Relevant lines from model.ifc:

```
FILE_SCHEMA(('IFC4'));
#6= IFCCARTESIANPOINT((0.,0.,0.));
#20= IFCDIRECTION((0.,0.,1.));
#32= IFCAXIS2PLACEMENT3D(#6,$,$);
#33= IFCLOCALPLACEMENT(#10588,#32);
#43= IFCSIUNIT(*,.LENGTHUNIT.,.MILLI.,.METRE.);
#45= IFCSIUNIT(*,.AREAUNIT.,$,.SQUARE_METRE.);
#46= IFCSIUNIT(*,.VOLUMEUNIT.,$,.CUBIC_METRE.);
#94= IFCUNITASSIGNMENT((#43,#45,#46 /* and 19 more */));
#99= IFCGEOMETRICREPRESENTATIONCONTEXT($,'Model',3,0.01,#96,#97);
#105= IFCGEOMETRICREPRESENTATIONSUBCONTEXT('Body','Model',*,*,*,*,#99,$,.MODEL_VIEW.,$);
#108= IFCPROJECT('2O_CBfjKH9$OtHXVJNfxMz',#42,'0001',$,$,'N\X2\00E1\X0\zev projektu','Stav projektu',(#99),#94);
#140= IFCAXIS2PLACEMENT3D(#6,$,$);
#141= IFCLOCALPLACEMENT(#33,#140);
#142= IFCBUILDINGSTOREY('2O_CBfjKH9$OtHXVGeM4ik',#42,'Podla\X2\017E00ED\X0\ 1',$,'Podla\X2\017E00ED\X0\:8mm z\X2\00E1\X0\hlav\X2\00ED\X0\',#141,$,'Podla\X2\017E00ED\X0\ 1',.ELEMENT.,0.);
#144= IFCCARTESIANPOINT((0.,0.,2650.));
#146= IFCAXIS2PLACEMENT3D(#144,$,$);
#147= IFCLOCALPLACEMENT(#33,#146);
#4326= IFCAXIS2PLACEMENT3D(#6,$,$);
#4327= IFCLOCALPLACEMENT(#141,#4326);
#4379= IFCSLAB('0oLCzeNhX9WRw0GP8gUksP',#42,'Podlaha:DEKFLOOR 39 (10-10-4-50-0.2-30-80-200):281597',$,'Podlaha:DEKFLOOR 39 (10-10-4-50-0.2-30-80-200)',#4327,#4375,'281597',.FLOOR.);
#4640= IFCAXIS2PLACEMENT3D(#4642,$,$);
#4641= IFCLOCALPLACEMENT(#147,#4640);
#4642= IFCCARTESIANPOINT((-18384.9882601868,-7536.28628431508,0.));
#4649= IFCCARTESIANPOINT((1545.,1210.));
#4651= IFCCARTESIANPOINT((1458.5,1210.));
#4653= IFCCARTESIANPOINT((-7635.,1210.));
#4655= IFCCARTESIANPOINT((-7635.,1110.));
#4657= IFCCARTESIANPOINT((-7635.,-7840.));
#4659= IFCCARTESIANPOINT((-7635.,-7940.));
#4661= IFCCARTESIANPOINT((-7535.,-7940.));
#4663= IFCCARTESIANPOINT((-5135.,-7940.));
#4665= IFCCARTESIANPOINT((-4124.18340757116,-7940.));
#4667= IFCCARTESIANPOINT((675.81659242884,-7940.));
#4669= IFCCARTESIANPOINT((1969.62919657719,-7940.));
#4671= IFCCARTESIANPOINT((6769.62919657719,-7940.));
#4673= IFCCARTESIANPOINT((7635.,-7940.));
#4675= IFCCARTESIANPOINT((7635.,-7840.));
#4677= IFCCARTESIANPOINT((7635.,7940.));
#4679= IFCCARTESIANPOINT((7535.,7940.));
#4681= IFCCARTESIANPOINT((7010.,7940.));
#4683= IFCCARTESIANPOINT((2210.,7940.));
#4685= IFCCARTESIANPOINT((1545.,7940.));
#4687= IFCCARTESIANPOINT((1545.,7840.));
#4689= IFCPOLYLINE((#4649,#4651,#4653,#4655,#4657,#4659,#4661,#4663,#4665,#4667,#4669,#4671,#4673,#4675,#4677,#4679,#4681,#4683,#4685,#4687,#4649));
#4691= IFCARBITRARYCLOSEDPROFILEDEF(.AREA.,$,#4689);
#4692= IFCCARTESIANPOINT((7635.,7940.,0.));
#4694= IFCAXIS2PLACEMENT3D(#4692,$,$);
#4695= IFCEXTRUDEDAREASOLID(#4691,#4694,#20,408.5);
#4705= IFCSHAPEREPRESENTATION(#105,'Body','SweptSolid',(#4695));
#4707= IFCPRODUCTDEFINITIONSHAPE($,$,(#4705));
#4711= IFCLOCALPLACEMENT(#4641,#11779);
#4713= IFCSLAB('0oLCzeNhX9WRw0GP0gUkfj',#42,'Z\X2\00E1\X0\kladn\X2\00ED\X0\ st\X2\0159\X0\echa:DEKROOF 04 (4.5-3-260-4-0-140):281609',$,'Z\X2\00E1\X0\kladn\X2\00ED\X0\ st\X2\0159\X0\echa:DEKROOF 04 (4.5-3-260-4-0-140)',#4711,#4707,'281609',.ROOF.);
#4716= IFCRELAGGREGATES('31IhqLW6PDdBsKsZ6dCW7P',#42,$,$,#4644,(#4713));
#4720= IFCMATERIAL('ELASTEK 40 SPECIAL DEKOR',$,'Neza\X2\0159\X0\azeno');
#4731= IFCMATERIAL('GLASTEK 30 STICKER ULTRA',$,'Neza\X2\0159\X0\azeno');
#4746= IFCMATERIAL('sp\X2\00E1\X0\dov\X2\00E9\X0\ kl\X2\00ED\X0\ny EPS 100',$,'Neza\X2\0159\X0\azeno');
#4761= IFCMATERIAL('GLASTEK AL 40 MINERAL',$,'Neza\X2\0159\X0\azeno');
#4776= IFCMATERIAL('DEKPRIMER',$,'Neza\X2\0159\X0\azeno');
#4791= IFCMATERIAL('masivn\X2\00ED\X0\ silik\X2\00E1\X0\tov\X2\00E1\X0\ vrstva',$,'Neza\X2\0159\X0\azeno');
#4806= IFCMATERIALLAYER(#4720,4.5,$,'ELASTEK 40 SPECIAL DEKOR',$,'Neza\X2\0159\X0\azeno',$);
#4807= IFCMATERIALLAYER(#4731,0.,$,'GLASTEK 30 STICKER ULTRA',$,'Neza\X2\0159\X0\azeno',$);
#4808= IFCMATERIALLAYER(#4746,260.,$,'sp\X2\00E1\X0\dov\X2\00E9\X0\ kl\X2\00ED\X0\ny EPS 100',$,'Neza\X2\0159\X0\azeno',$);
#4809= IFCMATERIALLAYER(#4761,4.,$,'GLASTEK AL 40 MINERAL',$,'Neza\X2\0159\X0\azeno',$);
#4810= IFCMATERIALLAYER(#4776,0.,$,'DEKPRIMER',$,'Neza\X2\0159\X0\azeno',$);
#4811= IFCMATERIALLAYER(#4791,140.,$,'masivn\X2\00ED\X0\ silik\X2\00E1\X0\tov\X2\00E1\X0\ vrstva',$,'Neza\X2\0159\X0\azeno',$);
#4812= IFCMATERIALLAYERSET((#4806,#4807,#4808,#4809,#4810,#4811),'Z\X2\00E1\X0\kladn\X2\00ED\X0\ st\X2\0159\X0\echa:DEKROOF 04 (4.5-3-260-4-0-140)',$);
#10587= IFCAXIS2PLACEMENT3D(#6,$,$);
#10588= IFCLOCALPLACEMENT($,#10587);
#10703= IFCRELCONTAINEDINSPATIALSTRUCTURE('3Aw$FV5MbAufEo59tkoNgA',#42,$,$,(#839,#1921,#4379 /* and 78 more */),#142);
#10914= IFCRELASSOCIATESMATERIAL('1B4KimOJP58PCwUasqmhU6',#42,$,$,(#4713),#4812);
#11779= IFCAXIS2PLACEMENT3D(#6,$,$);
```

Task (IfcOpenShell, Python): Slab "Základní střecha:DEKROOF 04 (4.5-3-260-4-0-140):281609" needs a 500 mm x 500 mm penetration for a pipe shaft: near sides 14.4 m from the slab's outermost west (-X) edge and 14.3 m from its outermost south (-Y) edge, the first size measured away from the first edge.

```python
import numpy as np
import ifcopenshell
import ifcopenshell.api.feature
import ifcopenshell.api.geometry
import ifcopenshell.api.root
import ifcopenshell.geom
import ifcopenshell.util.placement
import ifcopenshell.util.representation
import ifcopenshell.util.shape
import ifcopenshell.util.unit

model = ifcopenshell.open("model.ifc")
unit_scale = ifcopenshell.util.unit.calculate_unit_scale(model)
settings = ifcopenshell.geom.settings()


def volume(element):
    """Net volume in cubic metres, openings subtracted."""
    shape = ifcopenshell.geom.create_shape(settings, element)
    return ifcopenshell.util.shape.get_volume(shape.geometry)


slab = model.by_guid("0oLCzeNhX9WRw0GP0gUkfj")
before = volume(slab)

# Extent in the slab's own axes, in metres. The edges named are its -X and -Y sides.
slab_shape = ifcopenshell.geom.create_shape(settings, slab)
vertices = ifcopenshell.util.shape.get_vertices(slab_shape.geometry)
x_min, y_min, bottom = vertices.min(axis=0)
top = vertices[:, 2].max()

opening = ifcopenshell.api.root.create_entity(model, ifc_class="IfcOpeningElement", name="Pipe shaft opening", predefined_type="OPENING")
context = ifcopenshell.util.representation.get_context(model, "Model", "Body", "MODEL_VIEW")
width, depth = 0.5, 0.5
outline = [(0.0, 0.0), (width, 0.0), (width, depth), (0.0, depth), (0.0, 0.0)]
# Overshoot both faces by 50 mm so the cut is clean.
shape = ifcopenshell.api.geometry.add_slab_representation(
    model, context=context, depth=top - bottom + 0.1, polyline=outline
)
ifcopenshell.api.geometry.assign_representation(model, product=opening, representation=shape)

matrix = ifcopenshell.util.placement.get_local_placement(slab.ObjectPlacement)
matrix[:, 3] = matrix @ np.append(np.array([x_min + 14.4, y_min + 14.3, bottom - 0.05]) / unit_scale, 1.0)
ifcopenshell.api.geometry.edit_object_placement(model, product=opening, matrix=matrix, is_si=False)
ifcopenshell.api.feature.add_feature(model, feature=opening, element=slab)

after = volume(slab)

print(f"slab volume {before:.3f} -> {after:.3f} m3")

model.write("model_edited.ifc")
```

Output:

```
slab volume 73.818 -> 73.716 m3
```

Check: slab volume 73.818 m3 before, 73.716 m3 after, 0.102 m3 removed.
